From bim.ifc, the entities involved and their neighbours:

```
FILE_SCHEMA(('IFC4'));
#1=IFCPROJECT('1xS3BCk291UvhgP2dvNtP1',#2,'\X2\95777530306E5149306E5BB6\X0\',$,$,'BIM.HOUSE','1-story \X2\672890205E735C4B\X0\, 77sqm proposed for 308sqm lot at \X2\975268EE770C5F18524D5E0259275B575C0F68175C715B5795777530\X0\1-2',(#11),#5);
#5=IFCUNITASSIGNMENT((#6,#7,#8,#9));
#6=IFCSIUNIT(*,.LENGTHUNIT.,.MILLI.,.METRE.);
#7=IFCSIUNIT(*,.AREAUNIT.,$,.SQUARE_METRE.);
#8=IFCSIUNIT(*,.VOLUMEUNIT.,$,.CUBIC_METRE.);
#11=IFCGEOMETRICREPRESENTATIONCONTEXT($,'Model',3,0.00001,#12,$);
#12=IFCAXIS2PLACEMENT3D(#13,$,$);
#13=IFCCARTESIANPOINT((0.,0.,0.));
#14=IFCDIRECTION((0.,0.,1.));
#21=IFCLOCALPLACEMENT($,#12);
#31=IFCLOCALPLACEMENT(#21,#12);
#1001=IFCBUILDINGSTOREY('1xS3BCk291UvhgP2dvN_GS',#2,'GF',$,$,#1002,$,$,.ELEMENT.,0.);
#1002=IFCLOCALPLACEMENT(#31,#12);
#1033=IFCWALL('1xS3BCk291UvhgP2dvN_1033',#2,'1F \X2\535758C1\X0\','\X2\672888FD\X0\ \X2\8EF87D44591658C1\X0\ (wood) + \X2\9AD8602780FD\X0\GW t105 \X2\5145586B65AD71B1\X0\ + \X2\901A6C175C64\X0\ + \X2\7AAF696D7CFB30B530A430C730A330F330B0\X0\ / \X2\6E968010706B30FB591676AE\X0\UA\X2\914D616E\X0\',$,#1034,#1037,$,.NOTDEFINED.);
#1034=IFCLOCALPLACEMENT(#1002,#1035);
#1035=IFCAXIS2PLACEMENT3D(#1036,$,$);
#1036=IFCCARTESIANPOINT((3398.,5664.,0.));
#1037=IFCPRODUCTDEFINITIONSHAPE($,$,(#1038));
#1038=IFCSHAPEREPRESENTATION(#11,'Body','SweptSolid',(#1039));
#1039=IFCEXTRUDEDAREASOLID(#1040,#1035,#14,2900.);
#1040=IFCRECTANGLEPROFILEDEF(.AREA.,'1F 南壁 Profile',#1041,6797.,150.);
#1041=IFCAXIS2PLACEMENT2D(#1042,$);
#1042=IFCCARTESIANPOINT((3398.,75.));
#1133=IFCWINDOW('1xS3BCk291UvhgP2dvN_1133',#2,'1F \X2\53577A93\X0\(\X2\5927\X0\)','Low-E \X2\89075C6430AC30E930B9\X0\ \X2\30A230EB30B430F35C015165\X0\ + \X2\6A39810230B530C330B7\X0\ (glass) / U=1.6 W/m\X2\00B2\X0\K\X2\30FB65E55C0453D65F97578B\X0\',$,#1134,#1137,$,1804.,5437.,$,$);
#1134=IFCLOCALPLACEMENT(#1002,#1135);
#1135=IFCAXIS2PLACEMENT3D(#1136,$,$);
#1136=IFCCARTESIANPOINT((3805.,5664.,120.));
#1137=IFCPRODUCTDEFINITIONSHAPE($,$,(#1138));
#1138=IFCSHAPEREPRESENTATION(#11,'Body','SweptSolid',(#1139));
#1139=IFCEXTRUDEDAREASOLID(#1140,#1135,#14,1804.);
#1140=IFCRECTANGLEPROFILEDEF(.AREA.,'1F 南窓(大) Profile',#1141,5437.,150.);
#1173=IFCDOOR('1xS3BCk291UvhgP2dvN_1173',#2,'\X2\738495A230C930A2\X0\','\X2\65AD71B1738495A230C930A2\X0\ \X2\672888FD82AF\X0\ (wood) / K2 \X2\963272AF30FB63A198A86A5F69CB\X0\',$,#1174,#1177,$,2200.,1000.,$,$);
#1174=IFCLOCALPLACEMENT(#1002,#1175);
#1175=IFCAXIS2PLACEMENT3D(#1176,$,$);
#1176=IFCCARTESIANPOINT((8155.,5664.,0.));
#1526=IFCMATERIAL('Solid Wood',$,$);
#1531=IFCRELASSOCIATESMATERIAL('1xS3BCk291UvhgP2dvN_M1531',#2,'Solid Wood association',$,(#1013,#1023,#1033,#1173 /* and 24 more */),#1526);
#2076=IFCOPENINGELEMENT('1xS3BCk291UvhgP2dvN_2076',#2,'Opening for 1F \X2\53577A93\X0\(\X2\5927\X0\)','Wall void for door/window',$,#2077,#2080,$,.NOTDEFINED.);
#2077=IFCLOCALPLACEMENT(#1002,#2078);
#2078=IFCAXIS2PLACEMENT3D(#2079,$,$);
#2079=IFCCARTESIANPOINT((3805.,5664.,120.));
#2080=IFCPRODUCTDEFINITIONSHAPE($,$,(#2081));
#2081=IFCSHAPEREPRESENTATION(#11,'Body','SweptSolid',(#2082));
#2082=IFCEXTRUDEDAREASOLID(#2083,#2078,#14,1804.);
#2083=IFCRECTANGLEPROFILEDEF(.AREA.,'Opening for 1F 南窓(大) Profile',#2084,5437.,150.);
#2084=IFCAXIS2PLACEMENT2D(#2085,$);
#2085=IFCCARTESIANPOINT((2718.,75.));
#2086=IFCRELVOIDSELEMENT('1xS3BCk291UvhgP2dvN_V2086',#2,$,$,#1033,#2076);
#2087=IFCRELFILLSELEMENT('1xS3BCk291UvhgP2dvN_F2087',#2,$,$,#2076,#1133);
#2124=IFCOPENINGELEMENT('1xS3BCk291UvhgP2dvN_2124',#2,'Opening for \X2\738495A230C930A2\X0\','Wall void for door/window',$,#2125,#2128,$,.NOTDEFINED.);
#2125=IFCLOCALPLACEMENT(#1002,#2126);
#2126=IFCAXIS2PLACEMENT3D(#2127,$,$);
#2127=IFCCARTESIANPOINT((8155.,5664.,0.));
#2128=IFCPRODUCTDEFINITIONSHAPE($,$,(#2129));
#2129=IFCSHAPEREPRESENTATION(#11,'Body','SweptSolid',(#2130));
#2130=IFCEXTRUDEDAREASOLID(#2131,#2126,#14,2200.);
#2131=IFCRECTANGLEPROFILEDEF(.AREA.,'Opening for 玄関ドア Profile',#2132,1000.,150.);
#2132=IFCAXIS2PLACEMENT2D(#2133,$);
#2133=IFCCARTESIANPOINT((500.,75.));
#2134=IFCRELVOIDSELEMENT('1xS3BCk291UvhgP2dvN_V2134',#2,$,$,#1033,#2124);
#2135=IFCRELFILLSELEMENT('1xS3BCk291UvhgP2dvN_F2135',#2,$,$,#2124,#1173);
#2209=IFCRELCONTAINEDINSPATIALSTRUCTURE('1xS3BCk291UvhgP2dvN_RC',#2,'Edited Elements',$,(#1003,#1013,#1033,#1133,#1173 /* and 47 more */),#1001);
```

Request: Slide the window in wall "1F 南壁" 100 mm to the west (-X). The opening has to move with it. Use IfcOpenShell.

```python
import ifcopenshell
import ifcopenshell.api.geometry
import ifcopenshell.util.placement

model = ifcopenshell.open("bim.ifc")

window = model.by_id(1133)
opening = window.FillsVoids[0].RelatingOpeningElement
wall = opening.VoidsElements[0].RelatingBuildingElement

wall_matrix = ifcopenshell.util.placement.get_local_placement(wall.ObjectPlacement)
shift = wall_matrix[:3, 0] * -100.0
before = ifcopenshell.util.placement.get_local_placement(window.ObjectPlacement)[:3, 3].copy()

# The window is not placed relative to its opening, so move both.
for product in (opening, window):
    matrix = ifcopenshell.util.placement.get_local_placement(product.ObjectPlacement)
    matrix[:3, 3] += shift
    ifcopenshell.api.geometry.edit_object_placement(model, product=product, matrix=matrix, is_si=False)

after = ifcopenshell.util.placement.get_local_placement(window.ObjectPlacement)[:3, 3]
print("window moved by", (after - before).round(3) + 0.0)

model.write("bim_rev.ifc")
```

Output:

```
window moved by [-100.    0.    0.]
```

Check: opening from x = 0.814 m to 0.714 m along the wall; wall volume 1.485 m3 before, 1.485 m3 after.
